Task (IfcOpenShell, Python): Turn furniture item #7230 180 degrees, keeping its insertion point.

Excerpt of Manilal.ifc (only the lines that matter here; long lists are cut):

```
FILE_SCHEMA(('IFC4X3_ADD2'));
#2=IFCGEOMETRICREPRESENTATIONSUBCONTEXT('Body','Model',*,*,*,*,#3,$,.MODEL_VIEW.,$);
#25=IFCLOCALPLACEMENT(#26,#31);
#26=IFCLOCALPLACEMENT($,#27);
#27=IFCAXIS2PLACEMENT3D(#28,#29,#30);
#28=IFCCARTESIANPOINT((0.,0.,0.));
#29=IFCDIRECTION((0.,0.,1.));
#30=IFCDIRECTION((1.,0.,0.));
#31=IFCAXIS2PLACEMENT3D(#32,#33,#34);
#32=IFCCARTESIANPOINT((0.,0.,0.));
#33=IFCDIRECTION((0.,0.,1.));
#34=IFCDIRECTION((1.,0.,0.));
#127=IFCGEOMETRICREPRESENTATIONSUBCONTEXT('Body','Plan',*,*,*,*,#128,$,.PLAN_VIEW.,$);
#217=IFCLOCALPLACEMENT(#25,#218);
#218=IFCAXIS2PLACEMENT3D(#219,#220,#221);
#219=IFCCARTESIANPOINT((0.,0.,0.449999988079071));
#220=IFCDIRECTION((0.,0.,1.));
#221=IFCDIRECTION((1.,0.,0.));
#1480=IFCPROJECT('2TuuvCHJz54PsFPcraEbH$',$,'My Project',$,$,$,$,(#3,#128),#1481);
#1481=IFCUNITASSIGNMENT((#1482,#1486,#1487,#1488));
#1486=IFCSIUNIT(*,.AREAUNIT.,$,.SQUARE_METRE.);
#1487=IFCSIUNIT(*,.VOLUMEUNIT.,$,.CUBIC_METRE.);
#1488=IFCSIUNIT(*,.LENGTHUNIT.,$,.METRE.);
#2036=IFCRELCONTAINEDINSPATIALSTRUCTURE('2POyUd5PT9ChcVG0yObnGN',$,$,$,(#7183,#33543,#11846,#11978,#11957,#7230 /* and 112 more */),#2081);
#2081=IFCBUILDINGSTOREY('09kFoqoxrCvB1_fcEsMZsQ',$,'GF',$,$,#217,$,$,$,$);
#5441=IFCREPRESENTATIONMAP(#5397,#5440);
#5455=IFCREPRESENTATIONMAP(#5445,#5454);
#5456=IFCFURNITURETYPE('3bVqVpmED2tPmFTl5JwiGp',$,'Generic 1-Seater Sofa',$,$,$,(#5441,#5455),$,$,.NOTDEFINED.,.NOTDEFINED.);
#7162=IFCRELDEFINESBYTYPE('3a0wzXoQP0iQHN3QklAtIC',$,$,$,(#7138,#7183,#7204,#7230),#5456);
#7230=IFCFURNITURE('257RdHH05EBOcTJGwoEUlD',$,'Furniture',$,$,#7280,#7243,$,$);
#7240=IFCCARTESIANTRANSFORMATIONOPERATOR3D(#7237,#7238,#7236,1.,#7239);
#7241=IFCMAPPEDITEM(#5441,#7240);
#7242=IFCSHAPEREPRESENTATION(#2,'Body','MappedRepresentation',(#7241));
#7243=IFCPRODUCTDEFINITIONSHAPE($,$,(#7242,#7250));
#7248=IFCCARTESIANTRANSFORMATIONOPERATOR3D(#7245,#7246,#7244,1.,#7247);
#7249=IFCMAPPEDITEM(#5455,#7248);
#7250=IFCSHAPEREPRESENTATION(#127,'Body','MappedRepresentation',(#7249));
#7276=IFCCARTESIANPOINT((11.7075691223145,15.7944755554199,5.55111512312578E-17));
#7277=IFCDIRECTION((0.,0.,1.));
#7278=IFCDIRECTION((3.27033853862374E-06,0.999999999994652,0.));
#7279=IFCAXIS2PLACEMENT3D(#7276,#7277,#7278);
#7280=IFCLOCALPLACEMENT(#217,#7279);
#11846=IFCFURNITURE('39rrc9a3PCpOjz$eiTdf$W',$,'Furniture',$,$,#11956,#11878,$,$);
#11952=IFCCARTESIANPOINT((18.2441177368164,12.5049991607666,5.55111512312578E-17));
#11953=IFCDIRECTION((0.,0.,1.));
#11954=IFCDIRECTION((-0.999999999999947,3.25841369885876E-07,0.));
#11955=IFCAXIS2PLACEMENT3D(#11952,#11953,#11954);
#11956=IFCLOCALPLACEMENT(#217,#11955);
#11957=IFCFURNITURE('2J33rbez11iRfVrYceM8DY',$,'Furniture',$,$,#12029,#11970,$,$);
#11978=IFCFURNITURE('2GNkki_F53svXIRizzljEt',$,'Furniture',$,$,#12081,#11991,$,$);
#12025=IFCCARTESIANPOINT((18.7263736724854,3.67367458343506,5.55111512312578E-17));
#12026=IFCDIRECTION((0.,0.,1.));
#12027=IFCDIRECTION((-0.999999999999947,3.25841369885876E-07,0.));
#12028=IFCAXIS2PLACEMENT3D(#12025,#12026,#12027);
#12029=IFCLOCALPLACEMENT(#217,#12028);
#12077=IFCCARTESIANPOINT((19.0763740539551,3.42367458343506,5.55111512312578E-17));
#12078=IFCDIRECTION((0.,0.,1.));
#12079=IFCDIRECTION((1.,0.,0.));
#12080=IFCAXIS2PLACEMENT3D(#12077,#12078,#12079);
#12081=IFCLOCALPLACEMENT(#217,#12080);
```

```python
import ifcopenshell
import ifcopenshell.api.geometry
import ifcopenshell.util.placement

model = ifcopenshell.open("Manilal.ifc")

item = model.by_id(7230)
matrix = ifcopenshell.util.placement.get_local_placement(item.ObjectPlacement)
matrix = matrix @ ifcopenshell.util.placement.rotation(180, "Z")
ifcopenshell.api.geometry.edit_object_placement(model, product=item, matrix=matrix, is_si=False)

print(ifcopenshell.util.placement.get_local_placement(item.ObjectPlacement).round(3) + 0.0)

model.write("Manilal_v2.ifc")
```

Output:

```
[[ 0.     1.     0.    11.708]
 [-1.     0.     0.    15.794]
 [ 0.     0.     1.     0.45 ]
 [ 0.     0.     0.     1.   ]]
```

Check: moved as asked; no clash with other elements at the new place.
